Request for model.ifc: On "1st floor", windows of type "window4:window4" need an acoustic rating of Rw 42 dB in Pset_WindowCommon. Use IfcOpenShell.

First a look at what the model holds.

```python
import ifcopenshell
import ifcopenshell.util.element

model = ifcopenshell.open("model.ifc")
print(model.schema)
storey = next(s for s in model.by_type("IfcBuildingStorey") if s.Name == "1st floor")
windows = [e for e in ifcopenshell.util.element.get_decomposition(storey) if e.is_a("IfcWindow")]
seen = {}
for e in windows:
    element_type = ifcopenshell.util.element.get_type(e)
    key = (element_type.Name if element_type != e and element_type else None, ifcopenshell.util.element.get_pset(e, "Pset_WindowCommon", "AcousticRating"))
    seen[key] = seen.get(key, 0) + 1
for (name, value), count in sorted(seen.items(), key=str):
    print(count, "x", name, "|", value)
```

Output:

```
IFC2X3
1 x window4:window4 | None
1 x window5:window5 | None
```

```python
import ifcopenshell
import ifcopenshell.api.pset
import ifcopenshell.util.element

model = ifcopenshell.open("model.ifc")

storey = next(s for s in model.by_type("IfcBuildingStorey") if s.Name == "1st floor")
windows = [e for e in ifcopenshell.util.element.get_decomposition(storey) if e.is_a("IfcWindow")]

count = 0
for e in windows:
    element_type = ifcopenshell.util.element.get_type(e)
    if element_type in (None, e) or element_type.Name != "window4:window4":
        continue
    # add_pset returns the element's existing set when there is one.
    pset = ifcopenshell.api.pset.add_pset(model, product=e, name="Pset_WindowCommon")
    ifcopenshell.api.pset.edit_pset(model, pset=pset, properties={"AcousticRating": "Rw 42 dB"})
    count += 1

print(count, "windows updated")

model.write("model_edited.ifc")
```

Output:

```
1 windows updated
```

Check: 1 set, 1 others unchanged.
